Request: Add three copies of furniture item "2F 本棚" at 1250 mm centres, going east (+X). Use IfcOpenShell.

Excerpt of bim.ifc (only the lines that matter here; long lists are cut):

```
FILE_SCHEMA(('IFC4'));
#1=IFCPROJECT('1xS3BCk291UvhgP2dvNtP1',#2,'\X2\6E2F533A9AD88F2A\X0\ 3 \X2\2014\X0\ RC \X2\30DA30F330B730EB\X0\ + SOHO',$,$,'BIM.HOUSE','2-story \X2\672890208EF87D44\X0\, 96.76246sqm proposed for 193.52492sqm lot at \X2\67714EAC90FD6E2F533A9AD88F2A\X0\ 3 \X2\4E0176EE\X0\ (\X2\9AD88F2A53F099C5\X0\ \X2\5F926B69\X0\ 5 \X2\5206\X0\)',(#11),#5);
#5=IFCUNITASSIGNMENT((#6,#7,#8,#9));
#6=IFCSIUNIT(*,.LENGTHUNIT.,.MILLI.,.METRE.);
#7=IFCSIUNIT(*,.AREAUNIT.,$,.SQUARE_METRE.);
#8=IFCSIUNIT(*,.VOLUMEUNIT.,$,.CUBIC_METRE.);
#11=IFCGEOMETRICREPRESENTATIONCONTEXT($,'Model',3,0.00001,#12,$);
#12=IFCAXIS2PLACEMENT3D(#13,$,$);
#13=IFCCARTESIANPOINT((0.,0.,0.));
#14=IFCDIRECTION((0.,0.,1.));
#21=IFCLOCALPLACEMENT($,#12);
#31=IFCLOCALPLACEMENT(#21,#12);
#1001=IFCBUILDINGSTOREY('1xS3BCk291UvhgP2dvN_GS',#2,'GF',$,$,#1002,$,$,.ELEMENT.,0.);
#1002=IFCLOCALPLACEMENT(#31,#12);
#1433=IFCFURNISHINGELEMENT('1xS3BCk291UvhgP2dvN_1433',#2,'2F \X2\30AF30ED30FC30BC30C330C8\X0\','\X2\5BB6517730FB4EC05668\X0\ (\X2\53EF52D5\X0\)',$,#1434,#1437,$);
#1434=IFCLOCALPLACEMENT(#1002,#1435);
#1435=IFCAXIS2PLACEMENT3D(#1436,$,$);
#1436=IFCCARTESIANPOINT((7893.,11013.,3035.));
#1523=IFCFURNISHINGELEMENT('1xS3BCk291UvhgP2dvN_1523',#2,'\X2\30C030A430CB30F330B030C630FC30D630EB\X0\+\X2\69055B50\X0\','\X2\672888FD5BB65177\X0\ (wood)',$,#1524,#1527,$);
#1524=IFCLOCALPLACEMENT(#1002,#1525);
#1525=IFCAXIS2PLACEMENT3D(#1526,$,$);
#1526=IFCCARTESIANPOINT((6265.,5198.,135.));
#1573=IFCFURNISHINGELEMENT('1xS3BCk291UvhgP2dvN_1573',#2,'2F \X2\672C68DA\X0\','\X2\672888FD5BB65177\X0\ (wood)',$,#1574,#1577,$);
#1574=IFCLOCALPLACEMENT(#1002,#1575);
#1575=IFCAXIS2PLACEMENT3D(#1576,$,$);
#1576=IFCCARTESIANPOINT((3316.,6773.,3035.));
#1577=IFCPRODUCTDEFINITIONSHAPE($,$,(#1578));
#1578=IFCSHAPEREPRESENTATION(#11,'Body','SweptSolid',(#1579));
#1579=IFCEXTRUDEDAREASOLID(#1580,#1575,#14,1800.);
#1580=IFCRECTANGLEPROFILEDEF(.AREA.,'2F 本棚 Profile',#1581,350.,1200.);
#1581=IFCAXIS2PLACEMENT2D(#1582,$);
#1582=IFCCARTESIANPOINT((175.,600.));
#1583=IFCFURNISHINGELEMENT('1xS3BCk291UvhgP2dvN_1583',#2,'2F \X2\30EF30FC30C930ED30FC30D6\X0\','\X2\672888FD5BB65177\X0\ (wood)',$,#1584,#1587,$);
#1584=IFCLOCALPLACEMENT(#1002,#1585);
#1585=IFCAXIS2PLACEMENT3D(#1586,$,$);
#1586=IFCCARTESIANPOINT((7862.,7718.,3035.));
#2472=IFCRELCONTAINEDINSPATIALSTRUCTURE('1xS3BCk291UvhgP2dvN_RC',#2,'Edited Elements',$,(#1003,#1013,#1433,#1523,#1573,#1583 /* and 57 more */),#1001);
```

```python
import numpy as np
import ifcopenshell
import ifcopenshell.api.geometry
import ifcopenshell.api.root
import ifcopenshell.util.element
import ifcopenshell.util.placement

model = ifcopenshell.open("bim.ifc")


def reuse_history(source, copy):
    """copy_class also copies each property set's owner history, people and application; keep the originals."""
    for rel in copy.IsDefinedBy:
        if rel.is_a("IfcRelDefinesByProperties") and (history := rel.RelatingPropertyDefinition.OwnerHistory):
            rel.RelatingPropertyDefinition.OwnerHistory = source.OwnerHistory
            ifcopenshell.util.element.remove_deep2(model, history)


source = model.by_guid("1xS3BCk291UvhgP2dvN_1573")
base = ifcopenshell.util.placement.get_local_placement(source.ObjectPlacement)
step = np.array([1.0, 0.0, 0.0]) * 1250.0

for i in range(1, 4):
    copy = ifcopenshell.api.root.copy_class(model, product=source)
    copy.Representation = ifcopenshell.util.element.copy_deep(
        model, source.Representation, exclude=["IfcGeometricRepresentationContext", "IfcRepresentationMap"]
    )
    reuse_history(source, copy)
    matrix = base.copy()
    matrix[:3, 3] += i * step
    print("added at", matrix[:3, 3].round(3) + 0.0)
    ifcopenshell.api.geometry.edit_object_placement(model, product=copy, matrix=matrix, is_si=False)

model.write("bim_updated.ifc")
```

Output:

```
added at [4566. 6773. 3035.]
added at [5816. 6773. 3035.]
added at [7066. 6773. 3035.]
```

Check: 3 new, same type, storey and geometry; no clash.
